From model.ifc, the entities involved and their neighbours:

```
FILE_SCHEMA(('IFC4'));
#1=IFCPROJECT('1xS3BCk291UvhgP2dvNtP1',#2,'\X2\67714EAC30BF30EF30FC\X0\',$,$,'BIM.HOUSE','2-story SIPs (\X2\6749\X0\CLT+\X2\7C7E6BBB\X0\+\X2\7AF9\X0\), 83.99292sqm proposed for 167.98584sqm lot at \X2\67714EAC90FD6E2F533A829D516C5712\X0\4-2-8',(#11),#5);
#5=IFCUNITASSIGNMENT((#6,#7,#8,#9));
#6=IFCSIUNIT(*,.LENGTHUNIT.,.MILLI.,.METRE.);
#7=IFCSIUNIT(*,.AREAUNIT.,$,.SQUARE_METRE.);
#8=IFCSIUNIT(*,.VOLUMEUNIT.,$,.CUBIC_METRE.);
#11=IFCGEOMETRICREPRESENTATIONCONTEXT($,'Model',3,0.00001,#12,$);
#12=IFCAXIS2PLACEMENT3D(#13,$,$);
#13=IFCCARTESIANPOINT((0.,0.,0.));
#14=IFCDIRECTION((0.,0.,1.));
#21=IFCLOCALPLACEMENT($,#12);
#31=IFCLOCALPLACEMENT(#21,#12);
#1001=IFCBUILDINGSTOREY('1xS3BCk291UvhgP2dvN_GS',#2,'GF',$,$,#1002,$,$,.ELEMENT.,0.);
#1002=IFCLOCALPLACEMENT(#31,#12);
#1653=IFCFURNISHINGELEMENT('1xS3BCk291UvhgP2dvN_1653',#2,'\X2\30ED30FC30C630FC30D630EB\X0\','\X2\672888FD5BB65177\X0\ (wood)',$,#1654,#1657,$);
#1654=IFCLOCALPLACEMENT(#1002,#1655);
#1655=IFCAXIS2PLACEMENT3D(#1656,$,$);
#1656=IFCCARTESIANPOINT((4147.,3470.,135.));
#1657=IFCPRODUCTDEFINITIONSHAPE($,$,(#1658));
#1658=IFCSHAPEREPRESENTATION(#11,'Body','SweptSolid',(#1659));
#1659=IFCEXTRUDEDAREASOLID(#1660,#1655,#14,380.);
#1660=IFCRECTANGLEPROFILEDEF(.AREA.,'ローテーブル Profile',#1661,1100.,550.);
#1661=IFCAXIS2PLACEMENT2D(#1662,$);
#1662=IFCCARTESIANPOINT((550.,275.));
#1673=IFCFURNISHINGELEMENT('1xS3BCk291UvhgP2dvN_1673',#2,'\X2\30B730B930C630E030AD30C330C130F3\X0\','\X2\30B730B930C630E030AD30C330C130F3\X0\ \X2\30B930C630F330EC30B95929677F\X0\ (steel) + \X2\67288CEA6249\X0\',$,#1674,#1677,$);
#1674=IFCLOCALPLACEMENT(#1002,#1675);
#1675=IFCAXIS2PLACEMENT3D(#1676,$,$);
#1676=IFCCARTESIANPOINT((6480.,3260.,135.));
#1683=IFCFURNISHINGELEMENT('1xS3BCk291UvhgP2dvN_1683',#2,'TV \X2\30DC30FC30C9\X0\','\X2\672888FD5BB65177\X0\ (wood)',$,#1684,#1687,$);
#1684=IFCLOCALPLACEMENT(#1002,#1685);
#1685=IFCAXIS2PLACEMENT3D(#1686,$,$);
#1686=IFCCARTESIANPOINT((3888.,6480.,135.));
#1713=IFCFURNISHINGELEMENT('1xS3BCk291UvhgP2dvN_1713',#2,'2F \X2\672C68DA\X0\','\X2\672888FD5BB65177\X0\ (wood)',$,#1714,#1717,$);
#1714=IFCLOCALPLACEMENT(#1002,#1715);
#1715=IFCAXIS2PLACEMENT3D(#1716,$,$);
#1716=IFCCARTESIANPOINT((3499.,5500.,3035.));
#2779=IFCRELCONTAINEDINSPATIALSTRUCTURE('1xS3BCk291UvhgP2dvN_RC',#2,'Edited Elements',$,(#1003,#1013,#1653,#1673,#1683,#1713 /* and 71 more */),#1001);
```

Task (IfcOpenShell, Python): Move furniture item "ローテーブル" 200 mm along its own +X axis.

```python
import ifcopenshell
import ifcopenshell.api.geometry
import ifcopenshell.util.placement
import ifcopenshell.util.unit

model = ifcopenshell.open("model.ifc")
unit_scale = ifcopenshell.util.unit.calculate_unit_scale(model)

item = model.by_guid("1xS3BCk291UvhgP2dvN_1653")
matrix = ifcopenshell.util.placement.get_local_placement(item.ObjectPlacement)
matrix[:3, 3] += matrix[:3, 0] * 0.2 / unit_scale
ifcopenshell.api.geometry.edit_object_placement(model, product=item, matrix=matrix, is_si=False)

print(ifcopenshell.util.placement.get_local_placement(item.ObjectPlacement).round(3) + 0.0)

model.write("model_updated.ifc")
```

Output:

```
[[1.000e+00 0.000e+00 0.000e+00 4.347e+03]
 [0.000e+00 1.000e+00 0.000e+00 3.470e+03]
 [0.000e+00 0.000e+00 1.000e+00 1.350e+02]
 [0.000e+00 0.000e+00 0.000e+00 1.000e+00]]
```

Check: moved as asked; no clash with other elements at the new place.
